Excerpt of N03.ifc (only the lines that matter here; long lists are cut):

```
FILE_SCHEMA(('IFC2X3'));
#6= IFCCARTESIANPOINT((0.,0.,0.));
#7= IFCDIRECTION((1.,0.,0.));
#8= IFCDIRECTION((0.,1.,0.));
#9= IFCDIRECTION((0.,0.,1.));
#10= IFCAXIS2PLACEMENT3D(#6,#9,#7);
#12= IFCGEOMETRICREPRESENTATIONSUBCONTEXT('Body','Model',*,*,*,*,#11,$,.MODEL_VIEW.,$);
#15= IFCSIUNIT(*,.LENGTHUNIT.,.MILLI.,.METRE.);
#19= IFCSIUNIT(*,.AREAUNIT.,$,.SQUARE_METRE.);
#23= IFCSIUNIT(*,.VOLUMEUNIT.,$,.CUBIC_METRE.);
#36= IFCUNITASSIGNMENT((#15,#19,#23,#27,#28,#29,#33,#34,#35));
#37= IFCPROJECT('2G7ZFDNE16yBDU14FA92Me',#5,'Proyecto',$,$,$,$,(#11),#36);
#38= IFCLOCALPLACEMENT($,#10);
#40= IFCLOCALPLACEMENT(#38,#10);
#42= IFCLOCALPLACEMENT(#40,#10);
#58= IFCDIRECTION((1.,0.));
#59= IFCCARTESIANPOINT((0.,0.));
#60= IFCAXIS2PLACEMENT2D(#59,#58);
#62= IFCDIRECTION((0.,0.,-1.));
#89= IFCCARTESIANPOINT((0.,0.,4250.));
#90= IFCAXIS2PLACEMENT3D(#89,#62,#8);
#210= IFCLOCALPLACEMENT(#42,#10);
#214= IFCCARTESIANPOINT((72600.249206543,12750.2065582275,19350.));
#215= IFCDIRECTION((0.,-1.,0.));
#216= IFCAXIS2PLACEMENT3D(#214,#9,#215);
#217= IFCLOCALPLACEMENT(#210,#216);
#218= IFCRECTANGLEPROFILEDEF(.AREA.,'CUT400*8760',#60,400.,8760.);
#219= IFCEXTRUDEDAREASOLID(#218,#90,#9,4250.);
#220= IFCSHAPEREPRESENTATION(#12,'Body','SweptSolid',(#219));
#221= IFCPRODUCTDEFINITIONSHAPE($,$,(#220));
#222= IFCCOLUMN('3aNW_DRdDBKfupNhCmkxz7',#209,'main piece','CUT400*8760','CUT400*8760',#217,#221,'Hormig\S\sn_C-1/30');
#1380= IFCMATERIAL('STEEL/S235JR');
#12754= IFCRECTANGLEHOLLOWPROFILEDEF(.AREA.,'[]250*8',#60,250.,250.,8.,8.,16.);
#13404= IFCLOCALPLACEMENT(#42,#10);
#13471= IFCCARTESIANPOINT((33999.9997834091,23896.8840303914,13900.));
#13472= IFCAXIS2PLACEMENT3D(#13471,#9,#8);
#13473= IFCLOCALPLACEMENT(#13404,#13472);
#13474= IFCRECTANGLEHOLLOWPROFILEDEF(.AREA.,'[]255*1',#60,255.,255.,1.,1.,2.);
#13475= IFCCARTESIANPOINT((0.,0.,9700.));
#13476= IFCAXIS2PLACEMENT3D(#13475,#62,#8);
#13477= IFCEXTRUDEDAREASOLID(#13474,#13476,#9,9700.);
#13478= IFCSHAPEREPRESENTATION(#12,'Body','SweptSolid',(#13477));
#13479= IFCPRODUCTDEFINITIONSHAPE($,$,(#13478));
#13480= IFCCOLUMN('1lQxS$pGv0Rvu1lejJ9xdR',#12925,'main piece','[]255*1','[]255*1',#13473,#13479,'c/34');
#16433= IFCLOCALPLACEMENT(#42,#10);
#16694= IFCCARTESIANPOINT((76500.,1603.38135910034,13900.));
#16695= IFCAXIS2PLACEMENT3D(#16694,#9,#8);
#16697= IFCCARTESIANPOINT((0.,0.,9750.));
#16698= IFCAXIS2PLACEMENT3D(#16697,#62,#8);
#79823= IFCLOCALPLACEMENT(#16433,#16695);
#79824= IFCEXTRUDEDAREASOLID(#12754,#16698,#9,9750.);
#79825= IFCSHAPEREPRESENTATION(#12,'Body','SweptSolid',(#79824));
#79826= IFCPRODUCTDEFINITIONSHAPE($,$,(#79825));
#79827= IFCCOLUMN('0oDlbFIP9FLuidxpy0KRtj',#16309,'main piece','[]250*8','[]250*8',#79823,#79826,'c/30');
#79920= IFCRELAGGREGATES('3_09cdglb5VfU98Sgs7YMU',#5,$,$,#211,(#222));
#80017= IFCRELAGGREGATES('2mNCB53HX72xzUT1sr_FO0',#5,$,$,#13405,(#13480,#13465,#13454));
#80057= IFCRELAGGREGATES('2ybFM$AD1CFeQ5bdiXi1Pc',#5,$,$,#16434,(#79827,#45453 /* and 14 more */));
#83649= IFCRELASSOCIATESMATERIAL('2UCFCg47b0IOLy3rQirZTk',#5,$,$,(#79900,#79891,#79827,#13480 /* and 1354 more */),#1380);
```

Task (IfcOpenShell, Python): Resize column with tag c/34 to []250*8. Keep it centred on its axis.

```python
import ifcopenshell
import ifcopenshell.util.element
import ifcopenshell.util.representation

model = ifcopenshell.open("N03.ifc")

member = model.by_id(13480)
source = next(p for p in model.by_type("IfcRectangleHollowProfileDef") if p.ProfileName == "[]250*8")

body = ifcopenshell.util.representation.get_representation(member, "Model", "Body")
solid = body.Items[0]
old_profile = solid.SweptArea

# Copy the section's sizes but keep this member's own profile position.
profile = ifcopenshell.util.element.copy(model, source)
profile.Position = old_profile.Position
solid.SweptArea = profile
if not model.get_total_inverses(old_profile):
    ifcopenshell.util.element.remove_deep2(model, old_profile)
member.Description = member.Description.replace("[]255*1", "[]250*8")
member.ObjectType = member.ObjectType.replace("[]255*1", "[]250*8")

print(solid.SweptArea)

model.write("N03-out.ifc")
```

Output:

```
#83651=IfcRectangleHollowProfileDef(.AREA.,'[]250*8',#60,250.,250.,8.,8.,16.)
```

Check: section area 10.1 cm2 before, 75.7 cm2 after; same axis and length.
